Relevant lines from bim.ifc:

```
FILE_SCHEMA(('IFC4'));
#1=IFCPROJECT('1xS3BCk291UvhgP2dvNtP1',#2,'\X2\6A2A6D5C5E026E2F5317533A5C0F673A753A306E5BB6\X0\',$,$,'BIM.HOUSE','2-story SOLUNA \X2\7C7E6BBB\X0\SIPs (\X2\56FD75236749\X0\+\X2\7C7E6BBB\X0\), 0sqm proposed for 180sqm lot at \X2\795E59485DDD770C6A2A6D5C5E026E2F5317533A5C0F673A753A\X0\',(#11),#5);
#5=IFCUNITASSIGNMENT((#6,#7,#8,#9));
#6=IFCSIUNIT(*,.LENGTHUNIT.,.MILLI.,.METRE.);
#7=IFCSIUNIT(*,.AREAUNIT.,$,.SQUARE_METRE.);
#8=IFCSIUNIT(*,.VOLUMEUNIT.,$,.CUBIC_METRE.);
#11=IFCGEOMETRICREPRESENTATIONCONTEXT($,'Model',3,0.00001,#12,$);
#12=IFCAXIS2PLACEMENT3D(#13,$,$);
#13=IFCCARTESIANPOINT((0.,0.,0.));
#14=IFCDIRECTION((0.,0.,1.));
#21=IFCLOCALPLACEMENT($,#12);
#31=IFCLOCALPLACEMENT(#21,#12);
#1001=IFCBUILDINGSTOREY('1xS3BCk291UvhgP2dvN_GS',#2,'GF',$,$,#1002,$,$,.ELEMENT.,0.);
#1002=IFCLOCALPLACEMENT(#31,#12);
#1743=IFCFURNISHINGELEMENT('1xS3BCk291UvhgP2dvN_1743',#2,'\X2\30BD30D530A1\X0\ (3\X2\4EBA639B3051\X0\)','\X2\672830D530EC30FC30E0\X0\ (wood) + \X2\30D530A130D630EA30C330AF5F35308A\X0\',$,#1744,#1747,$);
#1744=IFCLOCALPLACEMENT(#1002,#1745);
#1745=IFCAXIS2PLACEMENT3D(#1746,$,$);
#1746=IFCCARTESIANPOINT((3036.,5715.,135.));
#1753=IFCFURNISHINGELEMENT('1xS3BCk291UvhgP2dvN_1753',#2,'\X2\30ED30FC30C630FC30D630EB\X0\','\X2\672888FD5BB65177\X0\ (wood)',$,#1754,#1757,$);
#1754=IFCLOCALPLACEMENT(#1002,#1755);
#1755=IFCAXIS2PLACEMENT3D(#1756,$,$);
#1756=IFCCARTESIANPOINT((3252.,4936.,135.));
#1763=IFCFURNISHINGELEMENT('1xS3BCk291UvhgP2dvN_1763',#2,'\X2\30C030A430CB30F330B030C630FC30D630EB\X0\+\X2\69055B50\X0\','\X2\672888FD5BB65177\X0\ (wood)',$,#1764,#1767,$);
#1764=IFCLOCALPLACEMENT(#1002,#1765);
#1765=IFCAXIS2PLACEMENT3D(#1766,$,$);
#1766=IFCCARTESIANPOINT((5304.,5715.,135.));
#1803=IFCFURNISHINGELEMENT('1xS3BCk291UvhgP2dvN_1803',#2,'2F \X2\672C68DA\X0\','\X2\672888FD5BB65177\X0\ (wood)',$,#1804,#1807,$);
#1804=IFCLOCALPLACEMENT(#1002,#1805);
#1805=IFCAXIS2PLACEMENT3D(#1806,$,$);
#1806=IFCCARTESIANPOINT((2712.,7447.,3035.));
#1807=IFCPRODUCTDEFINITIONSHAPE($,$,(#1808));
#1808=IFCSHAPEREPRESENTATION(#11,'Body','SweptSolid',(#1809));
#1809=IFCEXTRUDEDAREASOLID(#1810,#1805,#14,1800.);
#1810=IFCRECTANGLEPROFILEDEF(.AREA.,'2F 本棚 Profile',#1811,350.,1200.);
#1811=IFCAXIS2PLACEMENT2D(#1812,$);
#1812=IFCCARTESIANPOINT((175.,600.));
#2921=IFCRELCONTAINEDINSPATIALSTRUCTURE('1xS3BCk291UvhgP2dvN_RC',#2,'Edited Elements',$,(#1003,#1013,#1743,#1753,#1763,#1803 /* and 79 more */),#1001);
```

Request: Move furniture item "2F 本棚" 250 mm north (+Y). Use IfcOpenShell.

```python
import ifcopenshell
import ifcopenshell.api.geometry
import ifcopenshell.util.placement
import ifcopenshell.util.unit

model = ifcopenshell.open("bim.ifc")
unit_scale = ifcopenshell.util.unit.calculate_unit_scale(model)

item = model.by_guid("1xS3BCk291UvhgP2dvN_1803")
matrix = ifcopenshell.util.placement.get_local_placement(item.ObjectPlacement)
matrix[1, 3] += 0.25 / unit_scale
ifcopenshell.api.geometry.edit_object_placement(model, product=item, matrix=matrix, is_si=False)

print(ifcopenshell.util.placement.get_local_placement(item.ObjectPlacement).round(3) + 0.0)

model.write("bim_edited.ifc")
```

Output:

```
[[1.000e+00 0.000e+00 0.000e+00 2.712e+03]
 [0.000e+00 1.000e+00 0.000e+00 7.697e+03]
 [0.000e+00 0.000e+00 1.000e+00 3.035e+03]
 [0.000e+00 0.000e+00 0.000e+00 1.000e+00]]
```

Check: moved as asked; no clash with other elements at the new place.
